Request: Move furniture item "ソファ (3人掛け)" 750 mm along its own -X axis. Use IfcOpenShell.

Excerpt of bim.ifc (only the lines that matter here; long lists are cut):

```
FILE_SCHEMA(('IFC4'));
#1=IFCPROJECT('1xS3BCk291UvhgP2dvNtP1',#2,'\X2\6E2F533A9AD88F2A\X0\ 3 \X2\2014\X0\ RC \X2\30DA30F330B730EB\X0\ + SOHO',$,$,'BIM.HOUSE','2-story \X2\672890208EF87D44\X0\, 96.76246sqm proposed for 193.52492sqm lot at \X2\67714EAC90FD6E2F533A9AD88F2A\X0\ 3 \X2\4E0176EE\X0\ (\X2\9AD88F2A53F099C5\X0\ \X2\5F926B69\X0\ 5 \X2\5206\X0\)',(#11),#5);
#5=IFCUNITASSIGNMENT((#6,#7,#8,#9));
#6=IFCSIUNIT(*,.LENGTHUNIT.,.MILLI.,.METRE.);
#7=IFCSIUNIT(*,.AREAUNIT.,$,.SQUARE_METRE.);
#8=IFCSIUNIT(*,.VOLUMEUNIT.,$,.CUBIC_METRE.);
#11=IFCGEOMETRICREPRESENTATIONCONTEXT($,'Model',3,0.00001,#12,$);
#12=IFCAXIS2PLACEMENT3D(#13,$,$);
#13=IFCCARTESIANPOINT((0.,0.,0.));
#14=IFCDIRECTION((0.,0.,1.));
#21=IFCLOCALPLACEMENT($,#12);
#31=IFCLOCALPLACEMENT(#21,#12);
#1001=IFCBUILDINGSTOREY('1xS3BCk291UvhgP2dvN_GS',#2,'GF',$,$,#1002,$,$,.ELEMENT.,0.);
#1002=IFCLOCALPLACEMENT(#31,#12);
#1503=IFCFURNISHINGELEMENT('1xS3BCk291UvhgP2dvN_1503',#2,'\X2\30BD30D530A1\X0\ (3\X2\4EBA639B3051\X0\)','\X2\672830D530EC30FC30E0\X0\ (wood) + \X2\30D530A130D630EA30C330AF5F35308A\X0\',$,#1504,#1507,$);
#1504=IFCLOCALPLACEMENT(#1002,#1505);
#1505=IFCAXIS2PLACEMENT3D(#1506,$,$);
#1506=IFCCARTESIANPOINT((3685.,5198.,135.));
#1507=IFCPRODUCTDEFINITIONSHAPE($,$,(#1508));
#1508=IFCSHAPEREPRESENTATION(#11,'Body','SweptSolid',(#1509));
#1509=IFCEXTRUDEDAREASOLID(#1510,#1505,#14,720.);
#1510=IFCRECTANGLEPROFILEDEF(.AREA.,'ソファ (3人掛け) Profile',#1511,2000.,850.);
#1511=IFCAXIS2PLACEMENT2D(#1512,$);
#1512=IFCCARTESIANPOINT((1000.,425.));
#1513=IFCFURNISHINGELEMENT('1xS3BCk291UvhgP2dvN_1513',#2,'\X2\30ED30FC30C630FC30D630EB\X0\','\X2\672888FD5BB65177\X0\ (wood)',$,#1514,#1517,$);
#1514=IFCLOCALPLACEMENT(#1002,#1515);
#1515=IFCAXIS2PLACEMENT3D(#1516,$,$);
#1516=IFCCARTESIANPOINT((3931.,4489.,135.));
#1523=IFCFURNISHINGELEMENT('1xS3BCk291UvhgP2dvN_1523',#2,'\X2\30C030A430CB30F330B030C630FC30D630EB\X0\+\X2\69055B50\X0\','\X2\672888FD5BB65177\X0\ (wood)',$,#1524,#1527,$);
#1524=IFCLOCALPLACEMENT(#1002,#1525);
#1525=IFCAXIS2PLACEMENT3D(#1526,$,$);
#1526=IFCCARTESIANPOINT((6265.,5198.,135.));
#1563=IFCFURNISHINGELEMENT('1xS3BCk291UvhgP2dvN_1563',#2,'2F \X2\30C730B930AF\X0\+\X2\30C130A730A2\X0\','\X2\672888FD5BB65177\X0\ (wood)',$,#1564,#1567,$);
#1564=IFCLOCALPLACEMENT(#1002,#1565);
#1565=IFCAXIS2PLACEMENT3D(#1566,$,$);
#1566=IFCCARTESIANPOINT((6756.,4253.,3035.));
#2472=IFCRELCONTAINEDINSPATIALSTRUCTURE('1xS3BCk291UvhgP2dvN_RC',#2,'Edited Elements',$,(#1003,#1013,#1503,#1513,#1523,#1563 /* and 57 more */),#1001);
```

```python
import ifcopenshell
import ifcopenshell.api.geometry
import ifcopenshell.util.placement

model = ifcopenshell.open("bim.ifc")

item = model.by_guid("1xS3BCk291UvhgP2dvN_1503")
matrix = ifcopenshell.util.placement.get_local_placement(item.ObjectPlacement)
matrix[:3, 3] -= matrix[:3, 0] * 750.0
ifcopenshell.api.geometry.edit_object_placement(model, product=item, matrix=matrix, is_si=False)

print(ifcopenshell.util.placement.get_local_placement(item.ObjectPlacement).round(3) + 0.0)

model.write("bim_rev.ifc")
```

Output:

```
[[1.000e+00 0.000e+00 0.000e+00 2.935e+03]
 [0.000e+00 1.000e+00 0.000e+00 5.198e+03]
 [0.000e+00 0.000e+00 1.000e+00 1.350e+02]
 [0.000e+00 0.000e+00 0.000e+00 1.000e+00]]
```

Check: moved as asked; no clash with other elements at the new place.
